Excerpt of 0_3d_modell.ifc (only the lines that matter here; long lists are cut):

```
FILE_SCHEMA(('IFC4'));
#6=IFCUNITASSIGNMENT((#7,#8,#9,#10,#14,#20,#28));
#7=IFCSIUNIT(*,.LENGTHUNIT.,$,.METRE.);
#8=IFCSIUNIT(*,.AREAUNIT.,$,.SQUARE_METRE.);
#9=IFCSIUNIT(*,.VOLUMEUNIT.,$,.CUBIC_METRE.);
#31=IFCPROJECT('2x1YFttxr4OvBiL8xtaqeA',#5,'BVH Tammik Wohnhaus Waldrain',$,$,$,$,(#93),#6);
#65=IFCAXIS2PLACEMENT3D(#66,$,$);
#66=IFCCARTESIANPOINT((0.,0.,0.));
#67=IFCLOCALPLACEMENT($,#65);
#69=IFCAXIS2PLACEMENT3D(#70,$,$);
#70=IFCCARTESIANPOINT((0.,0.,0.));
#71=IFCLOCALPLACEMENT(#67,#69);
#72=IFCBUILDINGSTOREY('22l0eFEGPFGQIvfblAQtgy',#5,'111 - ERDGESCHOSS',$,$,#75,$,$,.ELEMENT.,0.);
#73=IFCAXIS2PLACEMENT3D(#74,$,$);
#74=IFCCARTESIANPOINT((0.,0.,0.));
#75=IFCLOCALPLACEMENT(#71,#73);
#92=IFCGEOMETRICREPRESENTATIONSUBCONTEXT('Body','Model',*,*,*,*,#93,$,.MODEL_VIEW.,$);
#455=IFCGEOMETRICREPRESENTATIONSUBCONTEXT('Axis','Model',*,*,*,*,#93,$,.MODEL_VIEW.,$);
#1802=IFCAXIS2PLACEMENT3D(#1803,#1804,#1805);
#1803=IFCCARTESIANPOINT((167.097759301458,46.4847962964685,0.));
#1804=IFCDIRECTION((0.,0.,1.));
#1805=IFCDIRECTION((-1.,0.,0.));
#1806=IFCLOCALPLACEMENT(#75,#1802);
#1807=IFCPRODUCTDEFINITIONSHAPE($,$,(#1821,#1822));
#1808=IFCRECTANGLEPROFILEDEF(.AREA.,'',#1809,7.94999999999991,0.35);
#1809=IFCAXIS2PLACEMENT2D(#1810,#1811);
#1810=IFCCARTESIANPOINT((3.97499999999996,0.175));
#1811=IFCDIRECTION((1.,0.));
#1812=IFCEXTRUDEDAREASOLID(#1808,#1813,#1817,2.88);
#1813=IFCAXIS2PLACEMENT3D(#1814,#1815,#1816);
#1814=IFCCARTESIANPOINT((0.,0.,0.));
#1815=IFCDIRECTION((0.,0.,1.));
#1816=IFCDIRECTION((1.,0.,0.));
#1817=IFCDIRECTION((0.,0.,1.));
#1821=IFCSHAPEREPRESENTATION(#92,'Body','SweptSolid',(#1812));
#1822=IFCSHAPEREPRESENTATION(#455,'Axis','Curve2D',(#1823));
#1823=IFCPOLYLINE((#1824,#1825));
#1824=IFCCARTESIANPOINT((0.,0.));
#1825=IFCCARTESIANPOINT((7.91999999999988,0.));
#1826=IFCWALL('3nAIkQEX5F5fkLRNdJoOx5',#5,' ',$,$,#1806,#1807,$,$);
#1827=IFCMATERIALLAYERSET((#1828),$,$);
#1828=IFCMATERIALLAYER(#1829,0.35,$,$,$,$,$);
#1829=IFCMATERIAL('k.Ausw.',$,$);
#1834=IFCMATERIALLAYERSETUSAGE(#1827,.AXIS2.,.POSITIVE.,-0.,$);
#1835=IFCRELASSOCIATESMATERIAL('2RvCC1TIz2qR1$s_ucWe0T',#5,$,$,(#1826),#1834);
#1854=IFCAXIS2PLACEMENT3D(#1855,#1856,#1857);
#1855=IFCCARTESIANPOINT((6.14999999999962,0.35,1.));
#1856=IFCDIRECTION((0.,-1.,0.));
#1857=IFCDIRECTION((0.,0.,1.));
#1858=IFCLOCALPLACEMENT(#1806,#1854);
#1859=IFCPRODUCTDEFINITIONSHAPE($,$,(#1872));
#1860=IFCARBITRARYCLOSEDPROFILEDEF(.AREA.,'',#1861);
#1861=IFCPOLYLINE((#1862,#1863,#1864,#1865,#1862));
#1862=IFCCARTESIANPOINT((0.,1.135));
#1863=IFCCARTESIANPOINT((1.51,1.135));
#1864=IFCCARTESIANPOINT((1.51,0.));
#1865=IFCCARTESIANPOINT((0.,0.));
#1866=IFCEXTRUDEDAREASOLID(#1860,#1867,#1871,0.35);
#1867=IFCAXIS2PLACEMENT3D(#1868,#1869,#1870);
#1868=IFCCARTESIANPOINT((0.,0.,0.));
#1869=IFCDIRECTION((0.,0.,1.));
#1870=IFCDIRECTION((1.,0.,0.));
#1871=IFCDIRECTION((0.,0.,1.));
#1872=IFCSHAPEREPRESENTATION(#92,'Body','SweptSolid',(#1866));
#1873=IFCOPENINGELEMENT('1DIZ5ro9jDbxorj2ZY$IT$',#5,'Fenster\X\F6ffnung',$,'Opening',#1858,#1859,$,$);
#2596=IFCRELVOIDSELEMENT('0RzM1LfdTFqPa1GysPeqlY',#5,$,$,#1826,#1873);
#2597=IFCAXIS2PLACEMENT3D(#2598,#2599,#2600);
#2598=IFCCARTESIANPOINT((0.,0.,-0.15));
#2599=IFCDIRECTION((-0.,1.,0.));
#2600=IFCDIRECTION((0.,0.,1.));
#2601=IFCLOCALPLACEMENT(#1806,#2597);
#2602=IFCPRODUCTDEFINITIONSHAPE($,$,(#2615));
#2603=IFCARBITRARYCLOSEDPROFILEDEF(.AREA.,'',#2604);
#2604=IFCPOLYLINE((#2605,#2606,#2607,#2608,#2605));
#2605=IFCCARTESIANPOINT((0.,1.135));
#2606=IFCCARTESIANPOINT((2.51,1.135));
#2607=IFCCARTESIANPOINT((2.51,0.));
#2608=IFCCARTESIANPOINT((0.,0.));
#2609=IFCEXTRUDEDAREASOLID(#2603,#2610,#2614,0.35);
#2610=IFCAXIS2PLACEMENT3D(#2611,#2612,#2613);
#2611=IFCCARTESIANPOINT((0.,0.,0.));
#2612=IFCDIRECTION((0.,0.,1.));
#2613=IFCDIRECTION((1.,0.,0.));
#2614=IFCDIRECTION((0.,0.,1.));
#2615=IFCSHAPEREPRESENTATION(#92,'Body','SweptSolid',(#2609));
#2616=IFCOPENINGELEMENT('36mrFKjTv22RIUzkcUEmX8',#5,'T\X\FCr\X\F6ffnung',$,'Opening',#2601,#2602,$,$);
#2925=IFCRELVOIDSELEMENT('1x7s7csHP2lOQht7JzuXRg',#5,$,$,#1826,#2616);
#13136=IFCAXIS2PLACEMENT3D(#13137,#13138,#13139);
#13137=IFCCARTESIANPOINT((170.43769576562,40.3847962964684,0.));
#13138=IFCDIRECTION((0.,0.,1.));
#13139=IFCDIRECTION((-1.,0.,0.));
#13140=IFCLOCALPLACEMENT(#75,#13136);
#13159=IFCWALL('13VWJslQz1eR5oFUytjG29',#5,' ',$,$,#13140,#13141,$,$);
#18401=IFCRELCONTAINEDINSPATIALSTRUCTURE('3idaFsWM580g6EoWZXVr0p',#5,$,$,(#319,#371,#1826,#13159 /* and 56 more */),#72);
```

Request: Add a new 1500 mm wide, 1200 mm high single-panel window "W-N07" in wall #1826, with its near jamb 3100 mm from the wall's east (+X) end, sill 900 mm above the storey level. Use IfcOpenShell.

```python
import numpy as np
import ifcopenshell
import ifcopenshell.api.feature
import ifcopenshell.api.geometry
import ifcopenshell.api.root
import ifcopenshell.api.spatial
import ifcopenshell.geom
import ifcopenshell.util.element
import ifcopenshell.util.placement
import ifcopenshell.util.representation
import ifcopenshell.util.shape
import ifcopenshell.util.unit

model = ifcopenshell.open("0_3d_modell.ifc")
unit_scale = ifcopenshell.util.unit.calculate_unit_scale(model)
settings = ifcopenshell.geom.settings()


def volume(element):
    """Net volume in cubic metres, openings subtracted."""
    shape = ifcopenshell.geom.create_shape(settings, element)
    return ifcopenshell.util.shape.get_volume(shape.geometry)


wall = model.by_id(1826)
storey = ifcopenshell.util.element.get_container(wall, ifc_class="IfcBuildingStorey")
context = ifcopenshell.util.representation.get_context(model, "Model", "Body", "MODEL_VIEW")
before = volume(wall)

width, height, from_end, sill = 1.5, 1.2, 3.1, 0.9  # metres

# The wall runs along its own X axis, and the end named is its -X end.
wall_shape = ifcopenshell.geom.create_shape(settings, wall)
x, y, z = ifcopenshell.util.shape.get_vertices(wall_shape.geometry).T
start = x.min() + from_end
face, thickness = float(y.min()), float(y.max() - y.min())
wall_matrix = ifcopenshell.util.placement.get_local_placement(wall.ObjectPlacement)
level = ifcopenshell.util.placement.get_local_placement(storey.ObjectPlacement)[2, 3]


def in_wall(x, y):
    """Placement at x, y metres in the wall's axes, at sill height."""
    matrix = wall_matrix.copy()
    matrix[:, 3] = wall_matrix @ np.array([x / unit_scale, y / unit_scale, 0.0, 1.0])
    matrix[2, 3] = level + sill / unit_scale
    return matrix


# Opening: a box that overshoots both wall faces by 50 mm.
opening = ifcopenshell.api.root.create_entity(model, ifc_class="IfcOpeningElement", predefined_type="OPENING")
box = ifcopenshell.api.geometry.add_wall_representation(
    model, context=context, length=width, height=height, thickness=thickness + 0.1
)
ifcopenshell.api.geometry.assign_representation(model, product=opening, representation=box)
ifcopenshell.api.geometry.edit_object_placement(model, product=opening, matrix=in_wall(start, face - 0.05), is_si=False)
ifcopenshell.api.feature.add_feature(model, feature=opening, element=wall)

window = ifcopenshell.api.root.create_entity(model, ifc_class="IfcWindow", name="W-N07", predefined_type="WINDOW")
window.OverallWidth, window.OverallHeight = width / unit_scale, height / unit_scale
window.PartitioningType = "SINGLE_PANEL"
body = ifcopenshell.api.geometry.add_window_representation(
    model,
    context=context,
    overall_width=window.OverallWidth,
    overall_height=window.OverallHeight,
    partition_type="SINGLE_PANEL",
)
ifcopenshell.api.geometry.assign_representation(model, product=window, representation=body)
ifcopenshell.api.spatial.assign_container(model, products=[window], relating_structure=storey)
ifcopenshell.api.feature.add_filling(model, opening=opening, element=window)

# Centre the window in the wall's thickness.
ifcopenshell.api.geometry.edit_object_placement(model, product=window, matrix=in_wall(start, face), is_si=False)
window_shape = ifcopenshell.geom.create_shape(settings, window)
depth = ifcopenshell.util.shape.get_vertices(window_shape.geometry)[:, 1]
offset = face + thickness / 2 - (depth.min() + depth.max()) / 2
ifcopenshell.api.geometry.edit_object_placement(model, product=window, matrix=in_wall(start, offset), is_si=False)

after = volume(wall)

print(f"wall volume {before:.3f} -> {after:.3f} m3")

model.write("0_3d_modell_edited.ifc")
```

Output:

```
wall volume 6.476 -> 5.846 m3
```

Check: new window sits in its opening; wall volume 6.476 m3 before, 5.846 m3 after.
